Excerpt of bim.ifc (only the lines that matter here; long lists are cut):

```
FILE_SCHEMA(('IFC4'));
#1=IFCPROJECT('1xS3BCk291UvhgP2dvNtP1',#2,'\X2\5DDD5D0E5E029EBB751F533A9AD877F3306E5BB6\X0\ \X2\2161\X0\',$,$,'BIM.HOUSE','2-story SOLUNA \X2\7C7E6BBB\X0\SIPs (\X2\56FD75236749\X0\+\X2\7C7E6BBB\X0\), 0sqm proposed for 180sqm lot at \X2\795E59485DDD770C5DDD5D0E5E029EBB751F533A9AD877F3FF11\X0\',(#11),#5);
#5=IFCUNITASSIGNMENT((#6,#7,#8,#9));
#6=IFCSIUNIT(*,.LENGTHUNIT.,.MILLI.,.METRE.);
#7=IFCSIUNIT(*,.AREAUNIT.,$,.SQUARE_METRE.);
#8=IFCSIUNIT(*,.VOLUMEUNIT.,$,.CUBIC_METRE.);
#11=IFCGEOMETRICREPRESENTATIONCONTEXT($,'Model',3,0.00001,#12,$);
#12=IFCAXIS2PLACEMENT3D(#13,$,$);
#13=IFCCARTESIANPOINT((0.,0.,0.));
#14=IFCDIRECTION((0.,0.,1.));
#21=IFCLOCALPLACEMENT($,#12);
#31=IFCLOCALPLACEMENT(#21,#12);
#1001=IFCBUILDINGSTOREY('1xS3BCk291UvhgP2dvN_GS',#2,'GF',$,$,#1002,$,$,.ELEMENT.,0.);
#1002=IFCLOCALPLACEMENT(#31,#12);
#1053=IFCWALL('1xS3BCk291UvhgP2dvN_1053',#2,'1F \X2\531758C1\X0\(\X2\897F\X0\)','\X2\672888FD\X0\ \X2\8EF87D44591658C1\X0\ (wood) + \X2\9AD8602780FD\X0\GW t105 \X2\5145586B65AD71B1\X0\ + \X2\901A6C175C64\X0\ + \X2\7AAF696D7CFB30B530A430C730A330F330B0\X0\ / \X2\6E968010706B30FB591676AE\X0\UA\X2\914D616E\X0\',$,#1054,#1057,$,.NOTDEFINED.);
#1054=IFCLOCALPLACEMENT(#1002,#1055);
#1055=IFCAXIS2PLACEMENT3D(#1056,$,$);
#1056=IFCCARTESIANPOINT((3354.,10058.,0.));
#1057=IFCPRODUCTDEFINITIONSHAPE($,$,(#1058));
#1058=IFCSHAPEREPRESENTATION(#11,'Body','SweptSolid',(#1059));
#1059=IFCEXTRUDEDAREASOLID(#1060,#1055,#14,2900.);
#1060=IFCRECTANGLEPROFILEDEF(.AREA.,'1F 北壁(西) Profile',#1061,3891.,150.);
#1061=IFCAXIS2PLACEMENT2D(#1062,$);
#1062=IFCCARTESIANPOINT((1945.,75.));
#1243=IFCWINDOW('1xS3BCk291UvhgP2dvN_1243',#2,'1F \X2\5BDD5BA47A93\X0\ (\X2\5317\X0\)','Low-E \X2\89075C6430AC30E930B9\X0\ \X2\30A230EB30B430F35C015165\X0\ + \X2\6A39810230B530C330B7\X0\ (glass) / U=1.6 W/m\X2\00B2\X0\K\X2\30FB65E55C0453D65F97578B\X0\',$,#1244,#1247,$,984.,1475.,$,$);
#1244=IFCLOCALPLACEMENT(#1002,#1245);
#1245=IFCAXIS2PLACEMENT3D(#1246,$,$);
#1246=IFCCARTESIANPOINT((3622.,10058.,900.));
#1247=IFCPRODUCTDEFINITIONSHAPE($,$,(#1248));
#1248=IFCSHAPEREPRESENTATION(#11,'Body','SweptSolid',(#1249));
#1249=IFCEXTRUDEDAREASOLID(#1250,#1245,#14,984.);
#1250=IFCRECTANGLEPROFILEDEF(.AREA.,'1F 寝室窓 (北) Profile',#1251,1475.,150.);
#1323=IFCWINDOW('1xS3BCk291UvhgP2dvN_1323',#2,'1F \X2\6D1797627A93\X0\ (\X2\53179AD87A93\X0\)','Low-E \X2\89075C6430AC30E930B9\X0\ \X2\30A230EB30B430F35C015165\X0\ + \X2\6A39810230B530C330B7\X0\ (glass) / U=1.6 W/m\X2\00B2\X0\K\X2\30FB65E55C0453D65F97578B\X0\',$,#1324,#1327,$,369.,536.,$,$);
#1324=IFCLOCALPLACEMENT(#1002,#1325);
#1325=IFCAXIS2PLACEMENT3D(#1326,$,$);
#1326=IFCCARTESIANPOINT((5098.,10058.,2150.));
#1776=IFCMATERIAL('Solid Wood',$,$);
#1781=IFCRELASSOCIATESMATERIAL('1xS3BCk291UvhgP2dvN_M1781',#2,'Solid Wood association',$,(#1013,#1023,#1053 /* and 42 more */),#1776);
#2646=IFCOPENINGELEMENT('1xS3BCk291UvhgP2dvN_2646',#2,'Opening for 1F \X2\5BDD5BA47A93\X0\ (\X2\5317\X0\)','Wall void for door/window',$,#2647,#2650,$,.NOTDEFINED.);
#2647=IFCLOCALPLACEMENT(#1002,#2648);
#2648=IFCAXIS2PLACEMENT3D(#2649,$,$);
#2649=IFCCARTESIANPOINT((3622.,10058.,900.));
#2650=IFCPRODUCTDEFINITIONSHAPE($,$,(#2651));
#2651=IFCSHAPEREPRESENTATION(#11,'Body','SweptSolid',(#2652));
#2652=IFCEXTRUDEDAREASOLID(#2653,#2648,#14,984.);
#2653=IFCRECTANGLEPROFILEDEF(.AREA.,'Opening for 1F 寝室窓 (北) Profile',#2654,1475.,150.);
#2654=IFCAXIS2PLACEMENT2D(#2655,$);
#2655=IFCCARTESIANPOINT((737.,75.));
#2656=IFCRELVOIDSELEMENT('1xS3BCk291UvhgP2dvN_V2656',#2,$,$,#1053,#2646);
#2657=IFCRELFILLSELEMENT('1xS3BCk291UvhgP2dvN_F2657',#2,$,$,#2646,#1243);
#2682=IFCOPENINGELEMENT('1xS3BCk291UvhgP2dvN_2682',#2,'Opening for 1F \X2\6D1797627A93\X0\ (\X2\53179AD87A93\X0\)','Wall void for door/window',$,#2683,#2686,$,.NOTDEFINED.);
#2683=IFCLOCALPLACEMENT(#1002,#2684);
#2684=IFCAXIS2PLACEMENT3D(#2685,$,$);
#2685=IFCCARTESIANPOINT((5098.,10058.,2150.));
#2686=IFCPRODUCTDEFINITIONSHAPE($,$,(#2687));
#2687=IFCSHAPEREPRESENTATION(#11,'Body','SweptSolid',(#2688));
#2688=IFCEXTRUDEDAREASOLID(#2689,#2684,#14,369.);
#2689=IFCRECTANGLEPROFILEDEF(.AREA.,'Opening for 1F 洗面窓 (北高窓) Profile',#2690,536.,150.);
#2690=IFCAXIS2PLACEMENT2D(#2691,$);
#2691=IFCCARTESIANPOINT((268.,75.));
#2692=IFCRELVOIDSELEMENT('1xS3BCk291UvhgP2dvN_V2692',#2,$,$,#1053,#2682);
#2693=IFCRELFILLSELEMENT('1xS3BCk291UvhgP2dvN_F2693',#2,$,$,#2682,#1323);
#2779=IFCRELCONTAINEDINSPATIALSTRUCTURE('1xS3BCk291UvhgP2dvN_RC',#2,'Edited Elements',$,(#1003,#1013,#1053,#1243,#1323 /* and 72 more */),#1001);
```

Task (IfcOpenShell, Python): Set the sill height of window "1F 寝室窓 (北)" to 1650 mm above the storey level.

```python
import numpy as np
import ifcopenshell
import ifcopenshell.api.geometry
import ifcopenshell.geom
import ifcopenshell.util.element
import ifcopenshell.util.placement
import ifcopenshell.util.shape
import ifcopenshell.util.unit

model = ifcopenshell.open("bim.ifc")
unit_scale = ifcopenshell.util.unit.calculate_unit_scale(model)

window = model.by_id(1243)
opening = window.FillsVoids[0].RelatingOpeningElement
storey = ifcopenshell.util.element.get_container(window, ifc_class="IfcBuildingStorey")
level = ifcopenshell.util.placement.get_local_placement(storey.ObjectPlacement)[2, 3]

# The opening's origin need not be at the sill, so measure its lowest point.
shape = ifcopenshell.geom.create_shape(ifcopenshell.geom.settings(), opening)
bottom = ifcopenshell.util.shape.get_shape_bottom_elevation(shape, shape.geometry) / unit_scale
dz = level + 1.65 / unit_scale - bottom

shift = np.array([0.0, 0.0, dz])
# The window is not placed relative to its opening, so move both.
for product in (opening, window):
    matrix = ifcopenshell.util.placement.get_local_placement(product.ObjectPlacement)
    matrix[:3, 3] += shift
    ifcopenshell.api.geometry.edit_object_placement(model, product=product, matrix=matrix, is_si=False)

print(f"moved by {dz * unit_scale:+.3f} m")

model.write("bim_rev.ifc")
```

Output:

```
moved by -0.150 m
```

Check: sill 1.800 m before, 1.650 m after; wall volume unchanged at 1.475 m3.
